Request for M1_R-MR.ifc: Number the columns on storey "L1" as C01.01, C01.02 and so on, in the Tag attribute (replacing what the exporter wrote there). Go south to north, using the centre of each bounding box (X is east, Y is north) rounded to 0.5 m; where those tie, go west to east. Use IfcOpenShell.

First a look at what the model holds.

```python
import ifcopenshell
import ifcopenshell.util.element
import ifcopenshell.util.placement

model = ifcopenshell.open("M1_R-MR.ifc")
print(model.schema)
storey = next(s for s in model.by_type("IfcBuildingStorey") if s.Name == "L1")
columns = [e for e in ifcopenshell.util.element.get_decomposition(storey) if e.is_a("IfcColumn")]
for e in sorted(columns, key=lambda e: e.id()):
    origin = ifcopenshell.util.placement.get_local_placement(e.ObjectPlacement)[:3, 3]
    print(e.id(), e.Tag, e.Name, origin.round(2) + 0.0, sep=" | ")
```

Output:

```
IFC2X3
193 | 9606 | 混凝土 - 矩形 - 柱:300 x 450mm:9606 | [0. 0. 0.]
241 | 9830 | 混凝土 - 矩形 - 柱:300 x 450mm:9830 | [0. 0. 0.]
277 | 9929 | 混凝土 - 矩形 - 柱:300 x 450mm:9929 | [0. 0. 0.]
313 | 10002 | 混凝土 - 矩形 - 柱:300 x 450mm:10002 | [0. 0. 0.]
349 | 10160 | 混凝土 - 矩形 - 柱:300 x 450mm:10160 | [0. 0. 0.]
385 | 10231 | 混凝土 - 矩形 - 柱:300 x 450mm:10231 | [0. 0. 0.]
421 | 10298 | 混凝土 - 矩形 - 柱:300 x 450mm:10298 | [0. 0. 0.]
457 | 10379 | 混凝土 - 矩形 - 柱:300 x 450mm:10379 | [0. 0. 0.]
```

```python
import ifcopenshell
import ifcopenshell.geom
import ifcopenshell.util.element
import ifcopenshell.util.shape

model = ifcopenshell.open("M1_R-MR.ifc")
settings = ifcopenshell.geom.settings()
settings.set("use-world-coords", True)


def centre(element):
    shape = ifcopenshell.geom.create_shape(settings, element)
    return ifcopenshell.util.shape.get_bbox_centroid(shape.geometry)


storey = next(s for s in model.by_type("IfcBuildingStorey") if s.Name == "L1")
columns = [e for e in ifcopenshell.util.element.get_decomposition(storey) if e.is_a("IfcColumn")]

# Insertion points can sit at a corner or the storey origin, so sort by the geometry (in metres).
centres = {e: centre(e) for e in columns}
columns.sort(key=lambda e: (round(centres[e][1] / 0.5), centres[e][0]))

for i, e in enumerate(columns, start=1):
    number = f"C01.{i:02d}"
    e.Tag = number
    print(e.id(), number)

model.write("M1_R-MR_updated.ifc")
```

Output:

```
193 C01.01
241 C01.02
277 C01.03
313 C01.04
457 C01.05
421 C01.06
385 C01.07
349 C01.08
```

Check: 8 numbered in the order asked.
